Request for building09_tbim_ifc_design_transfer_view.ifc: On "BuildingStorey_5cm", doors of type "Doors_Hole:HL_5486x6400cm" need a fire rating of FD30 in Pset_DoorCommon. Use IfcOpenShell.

First a look at what the model holds.

```python
import ifcopenshell
import ifcopenshell.util.element

model = ifcopenshell.open("building09_tbim_ifc_design_transfer_view.ifc")
print(model.schema)
storey = next(s for s in model.by_type("IfcBuildingStorey") if s.Name == "BuildingStorey_5cm")
doors = [e for e in ifcopenshell.util.element.get_decomposition(storey) if e.is_a("IfcDoor")]
seen = {}
for e in doors:
    element_type = ifcopenshell.util.element.get_type(e)
    key = (element_type.Name if element_type != e and element_type else None, ifcopenshell.util.element.get_pset(e, "Pset_DoorCommon", "FireRating"))
    seen[key] = seen.get(key, 0) + 1
for (name, value), count in sorted(seen.items(), key=str):
    print(count, "x", name, "|", value)
```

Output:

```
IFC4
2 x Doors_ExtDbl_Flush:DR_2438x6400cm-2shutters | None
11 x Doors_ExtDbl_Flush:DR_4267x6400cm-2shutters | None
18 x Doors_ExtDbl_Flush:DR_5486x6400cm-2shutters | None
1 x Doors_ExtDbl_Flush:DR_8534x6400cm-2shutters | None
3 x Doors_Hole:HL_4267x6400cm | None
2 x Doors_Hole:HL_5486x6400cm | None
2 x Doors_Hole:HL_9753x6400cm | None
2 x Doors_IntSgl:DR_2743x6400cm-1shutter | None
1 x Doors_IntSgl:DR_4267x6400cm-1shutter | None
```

```python
import ifcopenshell
import ifcopenshell.api.pset
import ifcopenshell.util.element

model = ifcopenshell.open("building09_tbim_ifc_design_transfer_view.ifc")

storey = next(s for s in model.by_type("IfcBuildingStorey") if s.Name == "BuildingStorey_5cm")
doors = [e for e in ifcopenshell.util.element.get_decomposition(storey) if e.is_a("IfcDoor")]

count = 0
for e in doors:
    element_type = ifcopenshell.util.element.get_type(e)
    if element_type in (None, e) or element_type.Name != "Doors_Hole:HL_5486x6400cm":
        continue
    # add_pset returns the element's existing set when there is one.
    pset = ifcopenshell.api.pset.add_pset(model, product=e, name="Pset_DoorCommon")
    ifcopenshell.api.pset.edit_pset(model, pset=pset, properties={"FireRating": "FD30"})
    count += 1

print(count, "doors updated")

model.write("building09_tbim_ifc_design_transfer_view_edited.ifc")
```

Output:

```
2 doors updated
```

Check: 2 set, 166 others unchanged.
